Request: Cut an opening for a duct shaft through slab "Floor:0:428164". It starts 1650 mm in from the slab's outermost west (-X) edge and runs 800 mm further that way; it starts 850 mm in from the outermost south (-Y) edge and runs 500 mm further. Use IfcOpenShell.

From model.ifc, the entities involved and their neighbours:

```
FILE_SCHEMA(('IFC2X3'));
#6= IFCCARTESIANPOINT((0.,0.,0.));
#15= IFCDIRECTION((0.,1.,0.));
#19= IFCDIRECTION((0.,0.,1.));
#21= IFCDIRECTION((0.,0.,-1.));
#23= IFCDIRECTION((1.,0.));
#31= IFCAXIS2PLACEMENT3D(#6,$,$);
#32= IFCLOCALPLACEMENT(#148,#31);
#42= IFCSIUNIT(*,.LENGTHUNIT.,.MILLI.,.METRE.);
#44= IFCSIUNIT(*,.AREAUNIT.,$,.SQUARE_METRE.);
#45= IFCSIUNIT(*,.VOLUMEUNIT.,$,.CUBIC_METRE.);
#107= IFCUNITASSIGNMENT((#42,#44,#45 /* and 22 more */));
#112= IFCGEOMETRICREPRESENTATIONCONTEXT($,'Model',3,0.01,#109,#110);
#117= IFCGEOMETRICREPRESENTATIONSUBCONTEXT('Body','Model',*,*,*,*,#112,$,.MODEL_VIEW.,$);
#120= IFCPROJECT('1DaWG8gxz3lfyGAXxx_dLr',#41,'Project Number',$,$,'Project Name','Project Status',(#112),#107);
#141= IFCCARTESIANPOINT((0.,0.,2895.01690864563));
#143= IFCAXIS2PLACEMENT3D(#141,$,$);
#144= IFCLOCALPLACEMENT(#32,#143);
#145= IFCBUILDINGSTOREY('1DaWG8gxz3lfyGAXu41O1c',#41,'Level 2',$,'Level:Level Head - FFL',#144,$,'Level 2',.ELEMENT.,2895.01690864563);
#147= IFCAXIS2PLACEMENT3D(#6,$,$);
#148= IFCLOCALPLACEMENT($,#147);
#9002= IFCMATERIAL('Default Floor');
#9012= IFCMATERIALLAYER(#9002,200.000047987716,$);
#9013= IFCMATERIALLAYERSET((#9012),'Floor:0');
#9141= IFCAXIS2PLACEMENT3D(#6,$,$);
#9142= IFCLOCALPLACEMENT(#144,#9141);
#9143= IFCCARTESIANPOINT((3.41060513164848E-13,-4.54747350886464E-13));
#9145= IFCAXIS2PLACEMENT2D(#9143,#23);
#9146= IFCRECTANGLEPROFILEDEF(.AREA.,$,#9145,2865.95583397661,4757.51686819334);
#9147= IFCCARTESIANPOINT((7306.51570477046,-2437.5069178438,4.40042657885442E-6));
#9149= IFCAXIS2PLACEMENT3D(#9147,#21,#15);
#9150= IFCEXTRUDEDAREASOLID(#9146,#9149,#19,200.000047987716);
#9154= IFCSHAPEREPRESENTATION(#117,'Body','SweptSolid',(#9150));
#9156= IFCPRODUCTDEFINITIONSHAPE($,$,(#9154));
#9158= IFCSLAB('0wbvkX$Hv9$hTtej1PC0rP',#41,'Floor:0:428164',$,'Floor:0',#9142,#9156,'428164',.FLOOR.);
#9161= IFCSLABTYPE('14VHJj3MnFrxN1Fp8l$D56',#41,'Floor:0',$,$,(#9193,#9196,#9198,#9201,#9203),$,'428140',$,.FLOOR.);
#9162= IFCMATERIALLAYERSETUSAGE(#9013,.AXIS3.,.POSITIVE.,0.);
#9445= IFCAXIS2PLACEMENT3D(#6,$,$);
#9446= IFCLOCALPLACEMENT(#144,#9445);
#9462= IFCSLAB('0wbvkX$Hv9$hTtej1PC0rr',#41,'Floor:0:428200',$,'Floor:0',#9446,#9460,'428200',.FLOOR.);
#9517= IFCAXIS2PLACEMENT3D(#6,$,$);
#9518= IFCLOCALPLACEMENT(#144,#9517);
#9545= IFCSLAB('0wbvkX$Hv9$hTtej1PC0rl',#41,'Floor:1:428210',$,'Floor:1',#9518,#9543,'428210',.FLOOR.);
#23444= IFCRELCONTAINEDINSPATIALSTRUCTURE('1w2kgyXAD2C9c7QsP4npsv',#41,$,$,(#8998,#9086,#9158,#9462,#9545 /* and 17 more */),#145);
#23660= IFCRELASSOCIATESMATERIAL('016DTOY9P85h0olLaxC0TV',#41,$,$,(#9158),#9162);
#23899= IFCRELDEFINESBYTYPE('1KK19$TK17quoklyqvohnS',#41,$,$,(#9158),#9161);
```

```python
import numpy as np
import ifcopenshell
import ifcopenshell.api.feature
import ifcopenshell.api.geometry
import ifcopenshell.api.root
import ifcopenshell.geom
import ifcopenshell.util.placement
import ifcopenshell.util.representation
import ifcopenshell.util.shape
import ifcopenshell.util.unit

model = ifcopenshell.open("model.ifc")
unit_scale = ifcopenshell.util.unit.calculate_unit_scale(model)
settings = ifcopenshell.geom.settings()


def volume(element):
    """Net volume in cubic metres, openings subtracted."""
    shape = ifcopenshell.geom.create_shape(settings, element)
    return ifcopenshell.util.shape.get_volume(shape.geometry)


slab = model.by_guid("0wbvkX$Hv9$hTtej1PC0rP")
before = volume(slab)

# Extent in the slab's own axes, in metres. The edges named are its -X and -Y sides.
slab_shape = ifcopenshell.geom.create_shape(settings, slab)
vertices = ifcopenshell.util.shape.get_vertices(slab_shape.geometry)
x_min, y_min, bottom = vertices.min(axis=0)
top = vertices[:, 2].max()

opening = ifcopenshell.api.root.create_entity(model, ifc_class="IfcOpeningElement", name="Duct shaft opening")
context = ifcopenshell.util.representation.get_context(model, "Model", "Body", "MODEL_VIEW")
width, depth = 0.8, 0.5
outline = [(0.0, 0.0), (width, 0.0), (width, depth), (0.0, depth), (0.0, 0.0)]
# Overshoot both faces by 50 mm so the cut is clean.
shape = ifcopenshell.api.geometry.add_slab_representation(
    model, context=context, depth=top - bottom + 0.1, polyline=outline
)
ifcopenshell.api.geometry.assign_representation(model, product=opening, representation=shape)

matrix = ifcopenshell.util.placement.get_local_placement(slab.ObjectPlacement)
matrix[:, 3] = matrix @ np.append(np.array([x_min + 1.65, y_min + 0.85, bottom - 0.05]) / unit_scale, 1.0)
ifcopenshell.api.geometry.edit_object_placement(model, product=opening, matrix=matrix, is_si=False)
ifcopenshell.api.feature.add_feature(model, feature=opening, element=slab)

after = volume(slab)

print(f"slab volume {before:.3f} -> {after:.3f} m3")

model.write("model_edited.ifc")
```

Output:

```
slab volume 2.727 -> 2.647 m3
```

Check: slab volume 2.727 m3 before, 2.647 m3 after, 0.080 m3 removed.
